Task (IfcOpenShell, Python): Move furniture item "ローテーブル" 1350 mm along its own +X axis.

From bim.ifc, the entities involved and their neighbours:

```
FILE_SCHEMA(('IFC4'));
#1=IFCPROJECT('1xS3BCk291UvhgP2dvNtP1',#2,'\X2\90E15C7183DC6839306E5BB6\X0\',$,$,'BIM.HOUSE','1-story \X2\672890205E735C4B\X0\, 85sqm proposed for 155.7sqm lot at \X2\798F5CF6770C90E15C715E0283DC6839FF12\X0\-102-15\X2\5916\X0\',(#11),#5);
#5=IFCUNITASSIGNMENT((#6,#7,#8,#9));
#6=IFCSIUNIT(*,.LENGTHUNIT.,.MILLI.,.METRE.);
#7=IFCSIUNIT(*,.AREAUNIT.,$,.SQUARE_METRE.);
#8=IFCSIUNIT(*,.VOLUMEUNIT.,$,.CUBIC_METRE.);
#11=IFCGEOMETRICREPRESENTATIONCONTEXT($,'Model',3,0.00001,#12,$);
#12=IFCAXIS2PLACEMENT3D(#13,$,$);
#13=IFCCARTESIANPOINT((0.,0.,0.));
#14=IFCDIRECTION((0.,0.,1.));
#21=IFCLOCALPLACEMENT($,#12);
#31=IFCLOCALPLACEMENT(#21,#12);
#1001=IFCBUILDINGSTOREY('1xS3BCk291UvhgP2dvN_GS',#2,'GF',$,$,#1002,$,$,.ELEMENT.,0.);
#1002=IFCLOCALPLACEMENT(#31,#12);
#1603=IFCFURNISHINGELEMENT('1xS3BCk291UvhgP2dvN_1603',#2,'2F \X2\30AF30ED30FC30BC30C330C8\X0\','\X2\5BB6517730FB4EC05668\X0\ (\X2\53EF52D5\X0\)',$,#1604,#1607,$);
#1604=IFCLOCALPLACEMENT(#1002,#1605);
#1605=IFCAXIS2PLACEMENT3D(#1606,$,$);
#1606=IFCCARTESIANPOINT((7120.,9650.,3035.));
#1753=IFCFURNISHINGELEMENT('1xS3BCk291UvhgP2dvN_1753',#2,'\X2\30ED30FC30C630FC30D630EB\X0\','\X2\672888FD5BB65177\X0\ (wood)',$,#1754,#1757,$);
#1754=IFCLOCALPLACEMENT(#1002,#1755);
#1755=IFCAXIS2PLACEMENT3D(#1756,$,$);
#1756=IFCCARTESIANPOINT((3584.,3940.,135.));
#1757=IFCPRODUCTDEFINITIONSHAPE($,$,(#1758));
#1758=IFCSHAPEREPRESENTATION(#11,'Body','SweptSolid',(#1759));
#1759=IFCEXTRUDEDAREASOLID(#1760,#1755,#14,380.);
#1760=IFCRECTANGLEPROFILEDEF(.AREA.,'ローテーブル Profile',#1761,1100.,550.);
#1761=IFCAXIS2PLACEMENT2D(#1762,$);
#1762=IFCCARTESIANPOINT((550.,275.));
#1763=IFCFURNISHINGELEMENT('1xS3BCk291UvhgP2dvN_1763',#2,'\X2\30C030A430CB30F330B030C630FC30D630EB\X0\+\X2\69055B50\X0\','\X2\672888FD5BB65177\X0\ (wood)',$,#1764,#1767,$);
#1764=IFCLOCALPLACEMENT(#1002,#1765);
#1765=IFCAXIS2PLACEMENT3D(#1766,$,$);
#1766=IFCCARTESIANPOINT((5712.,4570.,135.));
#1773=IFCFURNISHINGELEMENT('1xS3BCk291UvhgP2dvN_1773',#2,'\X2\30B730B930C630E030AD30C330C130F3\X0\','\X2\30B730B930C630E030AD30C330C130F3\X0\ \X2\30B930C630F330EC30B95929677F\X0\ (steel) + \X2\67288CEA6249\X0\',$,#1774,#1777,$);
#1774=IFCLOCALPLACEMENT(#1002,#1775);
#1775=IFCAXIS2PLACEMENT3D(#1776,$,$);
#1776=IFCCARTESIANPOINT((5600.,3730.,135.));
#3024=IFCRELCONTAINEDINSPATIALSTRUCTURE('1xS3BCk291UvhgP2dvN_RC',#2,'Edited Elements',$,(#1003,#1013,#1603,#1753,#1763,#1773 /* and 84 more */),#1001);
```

```python
import ifcopenshell
import ifcopenshell.api.geometry
import ifcopenshell.util.placement
import ifcopenshell.util.unit

model = ifcopenshell.open("bim.ifc")
unit_scale = ifcopenshell.util.unit.calculate_unit_scale(model)

item = model.by_guid("1xS3BCk291UvhgP2dvN_1753")
matrix = ifcopenshell.util.placement.get_local_placement(item.ObjectPlacement)
matrix[:3, 3] += matrix[:3, 0] * 1.35 / unit_scale
ifcopenshell.api.geometry.edit_object_placement(model, product=item, matrix=matrix, is_si=False)

print(ifcopenshell.util.placement.get_local_placement(item.ObjectPlacement).round(3) + 0.0)

model.write("bim_rev.ifc")
```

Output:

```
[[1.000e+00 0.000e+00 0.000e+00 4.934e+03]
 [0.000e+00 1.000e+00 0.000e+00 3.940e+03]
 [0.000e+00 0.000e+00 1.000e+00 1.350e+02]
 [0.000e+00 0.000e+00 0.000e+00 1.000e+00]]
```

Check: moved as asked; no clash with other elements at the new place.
